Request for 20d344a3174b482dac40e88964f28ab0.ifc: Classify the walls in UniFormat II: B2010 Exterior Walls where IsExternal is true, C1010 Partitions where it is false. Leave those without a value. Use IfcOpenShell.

First a look at what the model holds.

```python
import ifcopenshell
import ifcopenshell.util.element

model = ifcopenshell.open("20d344a3174b482dac40e88964f28ab0.ifc")
print(model.schema)
print("classifications:", [c.Name for c in model.by_type("IfcClassification")])
values = [ifcopenshell.util.element.get_pset(e, "Pset_WallCommon", "IsExternal") for e in model.by_type("IfcWall")]
for value in (True, False, None):
    print("IsExternal", value, values.count(value))
```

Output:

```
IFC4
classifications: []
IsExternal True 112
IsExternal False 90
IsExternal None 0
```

```python
import ifcopenshell
import ifcopenshell.api.classification
import ifcopenshell.util.element

model = ifcopenshell.open("20d344a3174b482dac40e88964f28ab0.ifc")

system = ifcopenshell.api.classification.add_classification(model, classification="UniFormat II")

walls = model.by_type("IfcWall")
external = {e: ifcopenshell.util.element.get_pset(e, "Pset_WallCommon", "IsExternal") for e in walls}
for flag, code, name in ((True, "B2010", "Exterior Walls"), (False, "C1010", "Partitions")):
    products = [e for e in walls if external[e] is flag]
    ifcopenshell.api.classification.add_reference(
        model, products=products, classification=system, identification=code, name=name
    )
    print(code, len(products))

model.write("20d344a3174b482dac40e88964f28ab0-out.ifc")
```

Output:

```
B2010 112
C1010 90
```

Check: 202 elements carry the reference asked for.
